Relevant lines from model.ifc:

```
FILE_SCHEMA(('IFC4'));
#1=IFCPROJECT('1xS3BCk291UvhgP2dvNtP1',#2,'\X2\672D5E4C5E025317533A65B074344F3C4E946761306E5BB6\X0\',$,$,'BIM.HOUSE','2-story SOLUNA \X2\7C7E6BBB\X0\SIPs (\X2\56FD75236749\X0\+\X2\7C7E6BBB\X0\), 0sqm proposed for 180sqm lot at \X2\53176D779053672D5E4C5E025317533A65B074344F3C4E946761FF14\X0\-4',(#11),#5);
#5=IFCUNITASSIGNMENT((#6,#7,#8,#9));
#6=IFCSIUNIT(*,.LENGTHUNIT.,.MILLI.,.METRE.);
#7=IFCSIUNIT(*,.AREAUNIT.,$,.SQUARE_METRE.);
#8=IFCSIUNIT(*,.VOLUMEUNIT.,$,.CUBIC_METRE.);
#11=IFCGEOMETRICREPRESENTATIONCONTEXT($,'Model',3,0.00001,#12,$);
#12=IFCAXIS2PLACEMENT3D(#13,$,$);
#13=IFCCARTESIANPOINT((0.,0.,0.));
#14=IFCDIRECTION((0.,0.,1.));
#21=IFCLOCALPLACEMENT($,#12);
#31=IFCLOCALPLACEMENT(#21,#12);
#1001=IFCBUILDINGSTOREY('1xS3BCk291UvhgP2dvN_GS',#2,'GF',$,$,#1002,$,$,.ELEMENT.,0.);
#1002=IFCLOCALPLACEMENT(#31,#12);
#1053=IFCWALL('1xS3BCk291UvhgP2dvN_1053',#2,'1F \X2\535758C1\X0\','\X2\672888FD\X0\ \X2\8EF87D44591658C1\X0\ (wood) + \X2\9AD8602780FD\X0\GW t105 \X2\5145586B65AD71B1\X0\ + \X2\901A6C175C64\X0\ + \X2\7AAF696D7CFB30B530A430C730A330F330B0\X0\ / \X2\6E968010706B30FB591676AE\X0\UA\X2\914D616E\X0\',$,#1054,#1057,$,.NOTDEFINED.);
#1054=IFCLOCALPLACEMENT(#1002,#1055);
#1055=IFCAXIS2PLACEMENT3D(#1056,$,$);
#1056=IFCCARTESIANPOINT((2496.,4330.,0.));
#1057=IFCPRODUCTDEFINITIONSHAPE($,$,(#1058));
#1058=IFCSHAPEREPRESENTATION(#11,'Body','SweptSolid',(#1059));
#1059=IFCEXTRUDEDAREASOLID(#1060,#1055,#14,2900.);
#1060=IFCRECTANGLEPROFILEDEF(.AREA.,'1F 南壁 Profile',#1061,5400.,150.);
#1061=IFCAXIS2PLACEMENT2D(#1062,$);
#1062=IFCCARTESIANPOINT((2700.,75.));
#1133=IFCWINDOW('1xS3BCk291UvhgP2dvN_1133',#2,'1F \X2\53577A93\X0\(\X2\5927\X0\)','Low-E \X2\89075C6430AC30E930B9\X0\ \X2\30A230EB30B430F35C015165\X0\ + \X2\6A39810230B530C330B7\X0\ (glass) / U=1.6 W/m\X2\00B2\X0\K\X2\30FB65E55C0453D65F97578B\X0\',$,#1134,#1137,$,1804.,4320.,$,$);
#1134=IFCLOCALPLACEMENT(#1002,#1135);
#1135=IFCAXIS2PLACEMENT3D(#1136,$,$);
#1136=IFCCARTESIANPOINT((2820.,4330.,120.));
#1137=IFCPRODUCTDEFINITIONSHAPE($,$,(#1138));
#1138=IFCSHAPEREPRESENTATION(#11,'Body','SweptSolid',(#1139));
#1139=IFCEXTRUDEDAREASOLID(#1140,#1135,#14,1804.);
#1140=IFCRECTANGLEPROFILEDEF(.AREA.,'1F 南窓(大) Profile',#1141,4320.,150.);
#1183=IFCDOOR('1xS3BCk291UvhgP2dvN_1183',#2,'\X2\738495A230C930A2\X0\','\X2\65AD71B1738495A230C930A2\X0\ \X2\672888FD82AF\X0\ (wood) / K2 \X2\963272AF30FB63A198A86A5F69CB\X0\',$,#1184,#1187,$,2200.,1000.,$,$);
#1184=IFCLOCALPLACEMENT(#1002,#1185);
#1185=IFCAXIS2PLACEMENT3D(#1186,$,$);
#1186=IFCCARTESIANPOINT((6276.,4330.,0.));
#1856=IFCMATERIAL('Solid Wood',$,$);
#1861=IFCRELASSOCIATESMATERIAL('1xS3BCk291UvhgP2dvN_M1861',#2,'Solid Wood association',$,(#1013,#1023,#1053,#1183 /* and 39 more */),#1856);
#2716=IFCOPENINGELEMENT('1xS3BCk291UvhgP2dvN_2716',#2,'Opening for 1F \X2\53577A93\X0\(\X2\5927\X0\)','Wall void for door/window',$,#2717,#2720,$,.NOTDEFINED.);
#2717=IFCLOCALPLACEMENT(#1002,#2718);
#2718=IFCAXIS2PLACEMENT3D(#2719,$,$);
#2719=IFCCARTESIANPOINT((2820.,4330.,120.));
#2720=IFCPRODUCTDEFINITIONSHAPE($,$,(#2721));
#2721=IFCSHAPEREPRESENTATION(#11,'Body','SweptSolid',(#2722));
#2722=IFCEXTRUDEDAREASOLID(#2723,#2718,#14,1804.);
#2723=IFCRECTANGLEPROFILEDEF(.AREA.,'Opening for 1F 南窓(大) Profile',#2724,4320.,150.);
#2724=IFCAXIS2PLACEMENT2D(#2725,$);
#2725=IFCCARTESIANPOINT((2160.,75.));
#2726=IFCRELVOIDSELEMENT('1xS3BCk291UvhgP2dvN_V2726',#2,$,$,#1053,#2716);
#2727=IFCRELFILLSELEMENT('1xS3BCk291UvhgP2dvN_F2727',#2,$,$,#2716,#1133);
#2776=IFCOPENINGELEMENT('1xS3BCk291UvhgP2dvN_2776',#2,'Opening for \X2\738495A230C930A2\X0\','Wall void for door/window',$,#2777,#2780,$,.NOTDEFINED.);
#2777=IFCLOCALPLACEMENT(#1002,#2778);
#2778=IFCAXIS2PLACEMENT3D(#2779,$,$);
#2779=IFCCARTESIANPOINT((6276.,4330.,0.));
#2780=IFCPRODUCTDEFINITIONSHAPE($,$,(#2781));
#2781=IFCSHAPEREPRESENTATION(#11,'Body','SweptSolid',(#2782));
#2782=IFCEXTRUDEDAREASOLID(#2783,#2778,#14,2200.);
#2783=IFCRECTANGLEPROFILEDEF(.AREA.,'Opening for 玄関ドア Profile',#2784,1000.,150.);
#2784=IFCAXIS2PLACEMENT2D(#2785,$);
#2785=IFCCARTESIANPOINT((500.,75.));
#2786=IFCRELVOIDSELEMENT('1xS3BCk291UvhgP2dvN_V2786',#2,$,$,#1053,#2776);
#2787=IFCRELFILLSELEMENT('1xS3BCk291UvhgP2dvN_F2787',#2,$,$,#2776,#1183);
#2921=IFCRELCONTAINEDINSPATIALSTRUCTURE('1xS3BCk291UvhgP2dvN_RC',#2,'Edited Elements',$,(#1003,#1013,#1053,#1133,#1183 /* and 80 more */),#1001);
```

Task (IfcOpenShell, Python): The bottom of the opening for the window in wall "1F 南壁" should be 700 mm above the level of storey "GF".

```python
import numpy as np
import ifcopenshell
import ifcopenshell.api.geometry
import ifcopenshell.geom
import ifcopenshell.util.element
import ifcopenshell.util.placement
import ifcopenshell.util.shape
import ifcopenshell.util.unit

model = ifcopenshell.open("model.ifc")
unit_scale = ifcopenshell.util.unit.calculate_unit_scale(model)

window = model.by_guid("1xS3BCk291UvhgP2dvN_1133")
opening = window.FillsVoids[0].RelatingOpeningElement
storey = ifcopenshell.util.element.get_container(window, ifc_class="IfcBuildingStorey")
level = ifcopenshell.util.placement.get_local_placement(storey.ObjectPlacement)[2, 3]

# The opening's origin need not be at the sill, so measure its lowest point.
shape = ifcopenshell.geom.create_shape(ifcopenshell.geom.settings(), opening)
bottom = ifcopenshell.util.shape.get_shape_bottom_elevation(shape, shape.geometry) / unit_scale
dz = level + 700.0 - bottom

shift = np.array([0.0, 0.0, dz])
# The window is not placed relative to its opening, so move both.
for product in (opening, window):
    matrix = ifcopenshell.util.placement.get_local_placement(product.ObjectPlacement)
    matrix[:3, 3] += shift
    ifcopenshell.api.geometry.edit_object_placement(model, product=product, matrix=matrix, is_si=False)

print(f"moved by {dz * unit_scale:+.3f} m")

model.write("model-out.ifc")
```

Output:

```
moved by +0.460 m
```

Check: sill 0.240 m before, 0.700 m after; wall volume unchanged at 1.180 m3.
